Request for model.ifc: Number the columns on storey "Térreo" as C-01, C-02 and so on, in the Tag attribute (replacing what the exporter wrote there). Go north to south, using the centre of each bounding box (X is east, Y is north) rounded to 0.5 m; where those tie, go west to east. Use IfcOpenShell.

First a look at what the model holds.

```python
import ifcopenshell
import ifcopenshell.util.element
import ifcopenshell.util.placement

model = ifcopenshell.open("model.ifc")
print(model.schema)
storey = next(s for s in model.by_type("IfcBuildingStorey") if s.Name == "Térreo")
columns = [e for e in ifcopenshell.util.element.get_decomposition(storey) if e.is_a("IfcColumn")]
for e in sorted(columns, key=lambda e: e.id()):
    origin = ifcopenshell.util.placement.get_local_placement(e.ObjectPlacement)[:3, 3]
    print(e.id(), e.Tag, e.Name, origin.round(2) + 0.0, sep=" | ")
```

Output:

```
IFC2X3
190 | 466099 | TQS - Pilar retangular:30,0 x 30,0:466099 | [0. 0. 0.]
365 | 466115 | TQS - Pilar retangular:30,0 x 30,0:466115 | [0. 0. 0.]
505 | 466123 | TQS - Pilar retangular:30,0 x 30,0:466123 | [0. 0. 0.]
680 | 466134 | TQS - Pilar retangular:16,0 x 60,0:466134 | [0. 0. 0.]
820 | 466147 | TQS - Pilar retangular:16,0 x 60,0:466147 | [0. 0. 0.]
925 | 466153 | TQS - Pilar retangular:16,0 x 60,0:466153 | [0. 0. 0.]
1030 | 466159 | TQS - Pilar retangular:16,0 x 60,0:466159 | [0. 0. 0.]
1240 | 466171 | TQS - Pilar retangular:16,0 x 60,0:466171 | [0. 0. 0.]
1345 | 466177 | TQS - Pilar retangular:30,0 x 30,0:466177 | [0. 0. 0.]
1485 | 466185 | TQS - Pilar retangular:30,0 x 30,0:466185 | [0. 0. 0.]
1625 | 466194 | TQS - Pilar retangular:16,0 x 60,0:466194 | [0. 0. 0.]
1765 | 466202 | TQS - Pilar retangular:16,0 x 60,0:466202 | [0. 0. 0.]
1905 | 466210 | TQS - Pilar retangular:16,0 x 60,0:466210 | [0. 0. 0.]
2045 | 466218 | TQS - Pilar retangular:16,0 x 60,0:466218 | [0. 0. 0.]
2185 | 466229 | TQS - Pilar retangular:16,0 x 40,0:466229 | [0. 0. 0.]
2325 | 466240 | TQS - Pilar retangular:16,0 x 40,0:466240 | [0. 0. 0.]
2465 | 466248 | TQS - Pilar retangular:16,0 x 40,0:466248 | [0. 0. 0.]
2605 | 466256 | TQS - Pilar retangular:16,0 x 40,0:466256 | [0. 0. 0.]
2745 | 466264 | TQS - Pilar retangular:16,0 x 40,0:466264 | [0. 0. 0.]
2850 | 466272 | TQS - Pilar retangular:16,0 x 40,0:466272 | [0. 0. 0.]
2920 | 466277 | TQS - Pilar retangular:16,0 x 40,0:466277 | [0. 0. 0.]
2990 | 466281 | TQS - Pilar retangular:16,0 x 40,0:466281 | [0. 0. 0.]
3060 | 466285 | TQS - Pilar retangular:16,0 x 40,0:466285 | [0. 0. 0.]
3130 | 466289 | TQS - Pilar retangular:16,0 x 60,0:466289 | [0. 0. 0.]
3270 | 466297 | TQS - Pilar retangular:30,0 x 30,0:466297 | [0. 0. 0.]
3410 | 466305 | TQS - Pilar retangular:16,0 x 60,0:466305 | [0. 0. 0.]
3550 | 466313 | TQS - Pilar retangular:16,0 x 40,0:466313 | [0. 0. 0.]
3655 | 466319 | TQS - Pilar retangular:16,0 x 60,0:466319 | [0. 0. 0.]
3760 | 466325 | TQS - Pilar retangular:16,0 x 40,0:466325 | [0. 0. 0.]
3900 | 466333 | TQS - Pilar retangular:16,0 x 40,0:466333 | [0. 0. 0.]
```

```python
import ifcopenshell
import ifcopenshell.geom
import ifcopenshell.util.element
import ifcopenshell.util.shape

model = ifcopenshell.open("model.ifc")
settings = ifcopenshell.geom.settings()
settings.set("use-world-coords", True)


def centre(element):
    shape = ifcopenshell.geom.create_shape(settings, element)
    return ifcopenshell.util.shape.get_bbox_centroid(shape.geometry)


storey = next(s for s in model.by_type("IfcBuildingStorey") if s.Name == "Térreo")
columns = [e for e in ifcopenshell.util.element.get_decomposition(storey) if e.is_a("IfcColumn")]

# Insertion points can sit at a corner or the storey origin, so sort by the geometry (in metres).
centres = {e: centre(e) for e in columns}
columns.sort(key=lambda e: (-round(centres[e][1] / 0.5), centres[e][0]))

for i, e in enumerate(columns, start=1):
    number = f"C-{i:02d}"
    e.Tag = number
    print(e.id(), number)

model.write("model_edited.ifc")
```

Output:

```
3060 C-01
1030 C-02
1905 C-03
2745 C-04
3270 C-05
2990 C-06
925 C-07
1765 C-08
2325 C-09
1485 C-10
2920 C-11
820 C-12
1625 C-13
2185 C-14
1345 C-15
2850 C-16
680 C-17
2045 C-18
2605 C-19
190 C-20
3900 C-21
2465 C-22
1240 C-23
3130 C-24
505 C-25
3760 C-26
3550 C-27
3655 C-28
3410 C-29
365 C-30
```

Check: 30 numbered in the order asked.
